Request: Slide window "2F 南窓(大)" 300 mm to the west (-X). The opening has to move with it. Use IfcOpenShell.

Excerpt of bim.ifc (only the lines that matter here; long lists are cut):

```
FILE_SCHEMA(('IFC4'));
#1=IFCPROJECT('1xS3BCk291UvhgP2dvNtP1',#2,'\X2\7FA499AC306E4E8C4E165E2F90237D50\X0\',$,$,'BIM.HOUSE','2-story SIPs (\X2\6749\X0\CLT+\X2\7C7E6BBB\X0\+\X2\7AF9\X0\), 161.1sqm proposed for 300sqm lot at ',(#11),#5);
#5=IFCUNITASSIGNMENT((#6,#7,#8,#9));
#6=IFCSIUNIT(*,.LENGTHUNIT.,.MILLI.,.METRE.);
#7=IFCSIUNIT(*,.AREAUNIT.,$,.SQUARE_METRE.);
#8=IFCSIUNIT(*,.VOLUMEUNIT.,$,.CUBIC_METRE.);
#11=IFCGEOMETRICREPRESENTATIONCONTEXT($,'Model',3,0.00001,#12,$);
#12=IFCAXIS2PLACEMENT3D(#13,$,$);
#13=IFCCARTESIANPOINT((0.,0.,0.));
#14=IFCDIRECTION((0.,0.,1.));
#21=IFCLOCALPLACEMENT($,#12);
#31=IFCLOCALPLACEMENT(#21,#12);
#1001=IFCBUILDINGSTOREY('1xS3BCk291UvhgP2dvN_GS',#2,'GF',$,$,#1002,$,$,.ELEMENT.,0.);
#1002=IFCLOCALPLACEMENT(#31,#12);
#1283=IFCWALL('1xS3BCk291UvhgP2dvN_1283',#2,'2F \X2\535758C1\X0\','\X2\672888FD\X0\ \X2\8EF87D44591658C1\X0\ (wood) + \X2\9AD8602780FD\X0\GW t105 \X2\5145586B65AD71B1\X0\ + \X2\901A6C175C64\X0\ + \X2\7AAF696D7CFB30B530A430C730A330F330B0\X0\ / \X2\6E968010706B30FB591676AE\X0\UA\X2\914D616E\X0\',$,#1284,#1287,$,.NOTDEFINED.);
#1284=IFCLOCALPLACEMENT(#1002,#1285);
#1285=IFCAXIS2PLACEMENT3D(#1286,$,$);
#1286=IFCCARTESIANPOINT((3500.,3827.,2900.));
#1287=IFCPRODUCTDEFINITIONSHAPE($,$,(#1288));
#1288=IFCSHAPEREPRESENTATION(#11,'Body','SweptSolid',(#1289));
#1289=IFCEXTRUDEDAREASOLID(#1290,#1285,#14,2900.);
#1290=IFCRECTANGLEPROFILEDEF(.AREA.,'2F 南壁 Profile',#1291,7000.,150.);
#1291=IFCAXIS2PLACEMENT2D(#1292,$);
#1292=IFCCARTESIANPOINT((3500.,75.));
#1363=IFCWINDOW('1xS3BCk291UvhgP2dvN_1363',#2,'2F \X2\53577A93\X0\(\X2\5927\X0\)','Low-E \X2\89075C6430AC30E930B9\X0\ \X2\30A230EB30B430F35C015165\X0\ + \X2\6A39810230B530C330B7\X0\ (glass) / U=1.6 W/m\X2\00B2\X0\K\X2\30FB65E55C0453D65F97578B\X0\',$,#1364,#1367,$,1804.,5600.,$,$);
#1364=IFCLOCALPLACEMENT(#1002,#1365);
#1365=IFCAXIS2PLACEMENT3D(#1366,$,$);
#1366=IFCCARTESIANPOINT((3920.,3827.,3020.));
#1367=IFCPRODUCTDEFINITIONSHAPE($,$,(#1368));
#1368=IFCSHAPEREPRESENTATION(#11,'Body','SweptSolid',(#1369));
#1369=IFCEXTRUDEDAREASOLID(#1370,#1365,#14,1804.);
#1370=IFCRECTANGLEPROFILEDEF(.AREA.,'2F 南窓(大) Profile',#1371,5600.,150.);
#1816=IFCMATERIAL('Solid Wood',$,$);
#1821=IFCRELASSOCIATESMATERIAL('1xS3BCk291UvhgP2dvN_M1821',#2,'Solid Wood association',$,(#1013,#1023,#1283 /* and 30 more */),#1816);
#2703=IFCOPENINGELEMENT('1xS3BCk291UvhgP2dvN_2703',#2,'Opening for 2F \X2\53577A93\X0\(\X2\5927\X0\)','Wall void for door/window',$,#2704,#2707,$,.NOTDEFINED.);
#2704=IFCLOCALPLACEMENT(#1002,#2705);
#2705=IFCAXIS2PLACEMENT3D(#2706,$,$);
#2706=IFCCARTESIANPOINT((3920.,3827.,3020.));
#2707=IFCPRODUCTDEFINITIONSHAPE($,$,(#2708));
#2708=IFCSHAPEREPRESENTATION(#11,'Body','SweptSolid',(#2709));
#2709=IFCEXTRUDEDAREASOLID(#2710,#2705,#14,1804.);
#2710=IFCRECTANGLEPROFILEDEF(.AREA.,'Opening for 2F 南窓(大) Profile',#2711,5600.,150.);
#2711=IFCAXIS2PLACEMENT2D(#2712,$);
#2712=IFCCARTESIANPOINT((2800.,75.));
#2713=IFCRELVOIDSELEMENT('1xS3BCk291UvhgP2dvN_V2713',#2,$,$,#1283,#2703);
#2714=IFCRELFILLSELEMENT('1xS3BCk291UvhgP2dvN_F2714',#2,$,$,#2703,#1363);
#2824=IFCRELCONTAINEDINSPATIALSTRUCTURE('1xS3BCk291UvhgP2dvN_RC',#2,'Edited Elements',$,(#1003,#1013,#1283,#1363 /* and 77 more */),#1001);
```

```python
import ifcopenshell
import ifcopenshell.api.geometry
import ifcopenshell.util.placement
import ifcopenshell.util.unit

model = ifcopenshell.open("bim.ifc")
unit_scale = ifcopenshell.util.unit.calculate_unit_scale(model)

window = model.by_id(1363)
opening = window.FillsVoids[0].RelatingOpeningElement
wall = opening.VoidsElements[0].RelatingBuildingElement

wall_matrix = ifcopenshell.util.placement.get_local_placement(wall.ObjectPlacement)
shift = wall_matrix[:3, 0] * -0.3 / unit_scale
before = ifcopenshell.util.placement.get_local_placement(window.ObjectPlacement)[:3, 3].copy()

# The window is not placed relative to its opening, so move both.
for product in (opening, window):
    matrix = ifcopenshell.util.placement.get_local_placement(product.ObjectPlacement)
    matrix[:3, 3] += shift
    ifcopenshell.api.geometry.edit_object_placement(model, product=product, matrix=matrix, is_si=False)

after = ifcopenshell.util.placement.get_local_placement(window.ObjectPlacement)[:3, 3]
print("window moved by", (after - before).round(3) + 0.0)

model.write("bim_edited.ifc")
```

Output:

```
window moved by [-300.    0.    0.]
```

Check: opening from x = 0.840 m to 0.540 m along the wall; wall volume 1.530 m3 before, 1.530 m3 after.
